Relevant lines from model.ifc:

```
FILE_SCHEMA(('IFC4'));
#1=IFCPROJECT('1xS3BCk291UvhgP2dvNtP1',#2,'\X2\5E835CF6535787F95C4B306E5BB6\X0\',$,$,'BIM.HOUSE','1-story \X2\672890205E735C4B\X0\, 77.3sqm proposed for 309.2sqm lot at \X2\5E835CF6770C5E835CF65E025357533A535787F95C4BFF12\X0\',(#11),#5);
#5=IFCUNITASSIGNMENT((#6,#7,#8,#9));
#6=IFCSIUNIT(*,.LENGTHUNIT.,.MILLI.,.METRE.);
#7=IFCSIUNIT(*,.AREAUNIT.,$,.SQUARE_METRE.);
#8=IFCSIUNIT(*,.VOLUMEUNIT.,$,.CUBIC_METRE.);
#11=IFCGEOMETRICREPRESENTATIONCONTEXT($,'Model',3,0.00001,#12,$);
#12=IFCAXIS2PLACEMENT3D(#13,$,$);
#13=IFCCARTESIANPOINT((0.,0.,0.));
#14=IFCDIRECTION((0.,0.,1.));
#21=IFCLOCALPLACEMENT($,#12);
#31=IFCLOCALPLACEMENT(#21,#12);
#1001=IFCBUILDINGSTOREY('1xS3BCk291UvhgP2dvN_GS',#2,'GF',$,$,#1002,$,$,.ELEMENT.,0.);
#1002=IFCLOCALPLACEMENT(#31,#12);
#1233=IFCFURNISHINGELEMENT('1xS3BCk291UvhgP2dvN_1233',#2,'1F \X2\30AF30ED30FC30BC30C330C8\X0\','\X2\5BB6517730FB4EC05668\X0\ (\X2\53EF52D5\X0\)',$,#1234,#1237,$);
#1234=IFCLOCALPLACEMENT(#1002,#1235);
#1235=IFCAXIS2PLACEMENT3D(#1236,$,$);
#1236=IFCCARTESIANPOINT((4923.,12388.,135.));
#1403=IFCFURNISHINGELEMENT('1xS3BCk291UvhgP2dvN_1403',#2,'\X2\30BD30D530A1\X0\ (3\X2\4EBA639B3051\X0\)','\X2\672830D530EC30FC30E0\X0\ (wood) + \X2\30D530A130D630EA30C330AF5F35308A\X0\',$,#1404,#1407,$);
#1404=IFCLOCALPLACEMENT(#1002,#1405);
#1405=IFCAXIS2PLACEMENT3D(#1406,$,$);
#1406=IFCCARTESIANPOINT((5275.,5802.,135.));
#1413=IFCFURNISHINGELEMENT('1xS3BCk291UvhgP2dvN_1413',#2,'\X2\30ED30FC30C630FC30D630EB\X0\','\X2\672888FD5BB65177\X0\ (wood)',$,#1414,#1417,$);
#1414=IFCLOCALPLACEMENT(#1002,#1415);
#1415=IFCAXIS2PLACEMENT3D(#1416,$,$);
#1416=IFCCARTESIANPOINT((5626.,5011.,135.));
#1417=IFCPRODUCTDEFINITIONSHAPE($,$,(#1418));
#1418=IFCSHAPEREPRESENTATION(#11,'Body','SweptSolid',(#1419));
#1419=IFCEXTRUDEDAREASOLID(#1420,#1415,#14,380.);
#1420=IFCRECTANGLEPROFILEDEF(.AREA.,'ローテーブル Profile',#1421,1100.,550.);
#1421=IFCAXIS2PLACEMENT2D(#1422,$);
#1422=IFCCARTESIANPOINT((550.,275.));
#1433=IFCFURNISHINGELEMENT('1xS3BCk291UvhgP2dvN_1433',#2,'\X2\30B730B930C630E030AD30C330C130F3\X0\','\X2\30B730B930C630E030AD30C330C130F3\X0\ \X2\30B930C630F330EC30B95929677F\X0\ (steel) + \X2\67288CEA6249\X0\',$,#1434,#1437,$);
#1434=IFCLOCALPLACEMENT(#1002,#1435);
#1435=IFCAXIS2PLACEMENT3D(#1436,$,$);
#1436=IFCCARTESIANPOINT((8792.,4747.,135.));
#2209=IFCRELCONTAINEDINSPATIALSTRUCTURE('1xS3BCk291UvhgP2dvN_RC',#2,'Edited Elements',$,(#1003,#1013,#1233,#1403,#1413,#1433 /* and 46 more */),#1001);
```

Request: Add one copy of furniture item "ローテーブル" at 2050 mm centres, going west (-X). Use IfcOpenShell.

```python
import numpy as np
import ifcopenshell
import ifcopenshell.api.geometry
import ifcopenshell.api.root
import ifcopenshell.util.element
import ifcopenshell.util.placement
import ifcopenshell.util.unit

model = ifcopenshell.open("model.ifc")
unit_scale = ifcopenshell.util.unit.calculate_unit_scale(model)


def reuse_history(source, copy):
    """copy_class also copies each property set's owner history, people and application; keep the originals."""
    for rel in copy.IsDefinedBy:
        if rel.is_a("IfcRelDefinesByProperties") and (history := rel.RelatingPropertyDefinition.OwnerHistory):
            rel.RelatingPropertyDefinition.OwnerHistory = source.OwnerHistory
            ifcopenshell.util.element.remove_deep2(model, history)


source = model.by_id(1413)
base = ifcopenshell.util.placement.get_local_placement(source.ObjectPlacement)
step = np.array([-1.0, 0.0, 0.0]) * 2.05 / unit_scale

for i in range(1, 2):
    copy = ifcopenshell.api.root.copy_class(model, product=source)
    copy.Representation = ifcopenshell.util.element.copy_deep(
        model, source.Representation, exclude=["IfcGeometricRepresentationContext", "IfcRepresentationMap"]
    )
    reuse_history(source, copy)
    matrix = base.copy()
    matrix[:3, 3] += i * step
    print("added at", matrix[:3, 3].round(3) + 0.0)
    ifcopenshell.api.geometry.edit_object_placement(model, product=copy, matrix=matrix, is_si=False)

model.write("model_updated.ifc")
```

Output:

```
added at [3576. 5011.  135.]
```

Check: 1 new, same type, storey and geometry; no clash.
